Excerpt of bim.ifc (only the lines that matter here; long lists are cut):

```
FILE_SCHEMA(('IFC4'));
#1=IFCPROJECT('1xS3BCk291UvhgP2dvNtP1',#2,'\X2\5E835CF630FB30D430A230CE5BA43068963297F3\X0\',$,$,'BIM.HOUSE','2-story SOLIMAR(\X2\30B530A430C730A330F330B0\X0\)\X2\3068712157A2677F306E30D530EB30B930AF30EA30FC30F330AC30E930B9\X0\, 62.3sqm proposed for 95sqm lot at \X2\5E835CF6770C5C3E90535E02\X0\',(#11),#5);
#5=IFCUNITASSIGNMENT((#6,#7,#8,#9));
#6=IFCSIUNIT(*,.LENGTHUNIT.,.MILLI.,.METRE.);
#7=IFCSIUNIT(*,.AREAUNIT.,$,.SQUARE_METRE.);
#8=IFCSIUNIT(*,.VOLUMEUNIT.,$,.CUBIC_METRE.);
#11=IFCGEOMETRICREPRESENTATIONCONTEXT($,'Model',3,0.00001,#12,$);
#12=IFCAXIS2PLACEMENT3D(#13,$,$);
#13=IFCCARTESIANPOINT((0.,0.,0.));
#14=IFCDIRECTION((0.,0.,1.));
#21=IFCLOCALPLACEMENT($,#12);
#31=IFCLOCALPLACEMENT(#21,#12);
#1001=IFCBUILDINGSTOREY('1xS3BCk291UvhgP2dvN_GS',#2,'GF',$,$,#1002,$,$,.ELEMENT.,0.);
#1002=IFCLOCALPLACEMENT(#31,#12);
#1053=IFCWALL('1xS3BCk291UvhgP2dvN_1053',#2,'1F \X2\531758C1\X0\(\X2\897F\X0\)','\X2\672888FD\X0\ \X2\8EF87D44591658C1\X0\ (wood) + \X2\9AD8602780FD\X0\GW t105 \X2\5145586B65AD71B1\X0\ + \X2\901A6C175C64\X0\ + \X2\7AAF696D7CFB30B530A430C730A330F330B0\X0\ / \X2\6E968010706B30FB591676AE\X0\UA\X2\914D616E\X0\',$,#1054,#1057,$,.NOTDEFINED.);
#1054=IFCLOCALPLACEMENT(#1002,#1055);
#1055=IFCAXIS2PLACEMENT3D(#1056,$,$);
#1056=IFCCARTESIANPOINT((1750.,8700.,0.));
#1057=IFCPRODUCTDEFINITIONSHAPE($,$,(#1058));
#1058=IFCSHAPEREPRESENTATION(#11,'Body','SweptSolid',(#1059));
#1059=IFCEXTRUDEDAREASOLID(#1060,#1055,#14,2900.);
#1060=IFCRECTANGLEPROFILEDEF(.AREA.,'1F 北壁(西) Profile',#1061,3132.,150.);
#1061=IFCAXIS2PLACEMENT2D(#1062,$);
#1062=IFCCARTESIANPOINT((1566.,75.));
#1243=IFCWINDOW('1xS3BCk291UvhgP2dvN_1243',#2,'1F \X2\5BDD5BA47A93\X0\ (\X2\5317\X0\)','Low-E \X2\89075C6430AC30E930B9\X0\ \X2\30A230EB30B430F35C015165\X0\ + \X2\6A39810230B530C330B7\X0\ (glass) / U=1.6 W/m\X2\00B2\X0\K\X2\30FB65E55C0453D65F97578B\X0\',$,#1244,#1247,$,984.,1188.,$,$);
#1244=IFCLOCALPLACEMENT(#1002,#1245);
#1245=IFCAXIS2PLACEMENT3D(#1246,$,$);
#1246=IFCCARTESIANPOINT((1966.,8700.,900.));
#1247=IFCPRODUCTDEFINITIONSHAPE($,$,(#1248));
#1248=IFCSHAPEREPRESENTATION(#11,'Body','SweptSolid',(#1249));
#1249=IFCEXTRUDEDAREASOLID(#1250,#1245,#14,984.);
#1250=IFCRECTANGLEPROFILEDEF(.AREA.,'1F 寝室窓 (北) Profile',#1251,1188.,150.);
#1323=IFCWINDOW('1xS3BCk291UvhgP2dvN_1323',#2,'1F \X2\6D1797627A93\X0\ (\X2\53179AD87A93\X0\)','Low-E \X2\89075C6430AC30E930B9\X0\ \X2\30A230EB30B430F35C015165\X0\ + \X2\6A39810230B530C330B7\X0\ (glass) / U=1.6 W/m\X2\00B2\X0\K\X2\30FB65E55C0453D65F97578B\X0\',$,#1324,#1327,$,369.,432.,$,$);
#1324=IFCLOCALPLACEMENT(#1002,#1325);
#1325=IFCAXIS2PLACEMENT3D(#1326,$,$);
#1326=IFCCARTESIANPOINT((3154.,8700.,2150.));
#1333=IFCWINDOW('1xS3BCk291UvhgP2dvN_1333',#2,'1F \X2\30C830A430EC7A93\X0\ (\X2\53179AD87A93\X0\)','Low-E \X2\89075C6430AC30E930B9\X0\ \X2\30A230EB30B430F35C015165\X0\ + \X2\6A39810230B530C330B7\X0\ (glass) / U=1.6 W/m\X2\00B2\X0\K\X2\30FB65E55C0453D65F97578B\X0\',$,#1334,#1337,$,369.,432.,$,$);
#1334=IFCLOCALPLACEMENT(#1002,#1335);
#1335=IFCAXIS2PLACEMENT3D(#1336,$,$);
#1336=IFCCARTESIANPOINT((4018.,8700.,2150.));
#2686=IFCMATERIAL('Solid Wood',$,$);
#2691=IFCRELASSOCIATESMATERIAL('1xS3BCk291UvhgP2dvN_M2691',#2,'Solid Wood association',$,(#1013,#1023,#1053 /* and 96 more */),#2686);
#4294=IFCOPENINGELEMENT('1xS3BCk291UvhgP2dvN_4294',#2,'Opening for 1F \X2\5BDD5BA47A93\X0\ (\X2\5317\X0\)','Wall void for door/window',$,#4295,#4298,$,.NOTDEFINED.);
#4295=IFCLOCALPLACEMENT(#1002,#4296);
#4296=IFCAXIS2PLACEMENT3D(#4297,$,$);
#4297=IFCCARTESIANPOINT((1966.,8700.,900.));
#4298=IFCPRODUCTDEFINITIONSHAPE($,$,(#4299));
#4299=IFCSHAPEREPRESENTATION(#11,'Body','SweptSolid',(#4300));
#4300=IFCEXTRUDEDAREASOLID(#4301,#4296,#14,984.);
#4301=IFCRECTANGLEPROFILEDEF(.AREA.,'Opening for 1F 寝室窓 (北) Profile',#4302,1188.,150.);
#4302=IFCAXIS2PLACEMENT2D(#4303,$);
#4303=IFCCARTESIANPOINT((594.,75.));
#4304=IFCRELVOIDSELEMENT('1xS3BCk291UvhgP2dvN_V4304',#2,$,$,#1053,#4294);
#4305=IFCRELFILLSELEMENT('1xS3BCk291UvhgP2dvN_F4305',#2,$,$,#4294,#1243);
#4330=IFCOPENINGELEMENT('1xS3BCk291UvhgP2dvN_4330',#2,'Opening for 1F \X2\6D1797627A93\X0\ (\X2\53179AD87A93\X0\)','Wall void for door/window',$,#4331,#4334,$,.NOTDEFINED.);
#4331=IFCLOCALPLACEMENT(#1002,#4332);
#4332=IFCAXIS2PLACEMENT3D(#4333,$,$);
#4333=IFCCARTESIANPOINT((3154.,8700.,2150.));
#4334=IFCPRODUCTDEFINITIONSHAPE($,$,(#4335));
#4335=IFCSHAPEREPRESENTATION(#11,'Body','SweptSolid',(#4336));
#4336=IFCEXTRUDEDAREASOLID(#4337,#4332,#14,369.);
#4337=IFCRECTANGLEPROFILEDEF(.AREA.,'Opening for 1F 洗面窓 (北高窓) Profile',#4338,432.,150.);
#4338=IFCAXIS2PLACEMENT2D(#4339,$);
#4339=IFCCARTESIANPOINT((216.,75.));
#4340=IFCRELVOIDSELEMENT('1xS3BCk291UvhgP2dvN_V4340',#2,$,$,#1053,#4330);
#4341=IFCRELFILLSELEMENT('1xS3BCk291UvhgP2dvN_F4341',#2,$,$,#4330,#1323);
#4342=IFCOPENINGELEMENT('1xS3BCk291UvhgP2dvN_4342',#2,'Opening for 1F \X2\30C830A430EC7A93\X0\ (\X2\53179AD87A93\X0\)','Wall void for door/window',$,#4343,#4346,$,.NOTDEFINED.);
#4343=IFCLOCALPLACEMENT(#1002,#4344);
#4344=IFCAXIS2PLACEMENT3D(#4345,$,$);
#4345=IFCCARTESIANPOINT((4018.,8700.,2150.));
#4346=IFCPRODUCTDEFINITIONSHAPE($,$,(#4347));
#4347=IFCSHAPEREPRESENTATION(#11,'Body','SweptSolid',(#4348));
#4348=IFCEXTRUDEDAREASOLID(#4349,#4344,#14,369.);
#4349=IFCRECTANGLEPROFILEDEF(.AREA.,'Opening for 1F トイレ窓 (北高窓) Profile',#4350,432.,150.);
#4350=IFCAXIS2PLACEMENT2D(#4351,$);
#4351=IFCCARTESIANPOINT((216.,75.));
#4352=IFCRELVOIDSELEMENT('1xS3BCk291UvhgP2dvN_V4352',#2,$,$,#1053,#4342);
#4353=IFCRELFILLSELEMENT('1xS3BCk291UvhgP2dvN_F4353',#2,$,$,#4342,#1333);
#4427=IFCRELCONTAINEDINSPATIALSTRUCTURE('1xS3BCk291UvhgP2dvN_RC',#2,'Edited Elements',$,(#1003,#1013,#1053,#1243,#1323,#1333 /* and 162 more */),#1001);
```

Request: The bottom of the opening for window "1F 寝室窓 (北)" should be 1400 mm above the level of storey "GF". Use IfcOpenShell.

```python
import numpy as np
import ifcopenshell
import ifcopenshell.api.geometry
import ifcopenshell.geom
import ifcopenshell.util.element
import ifcopenshell.util.placement
import ifcopenshell.util.shape
import ifcopenshell.util.unit

model = ifcopenshell.open("bim.ifc")
unit_scale = ifcopenshell.util.unit.calculate_unit_scale(model)

window = model.by_guid("1xS3BCk291UvhgP2dvN_1243")
opening = window.FillsVoids[0].RelatingOpeningElement
storey = ifcopenshell.util.element.get_container(window, ifc_class="IfcBuildingStorey")
level = ifcopenshell.util.placement.get_local_placement(storey.ObjectPlacement)[2, 3]

# The opening's origin need not be at the sill, so measure its lowest point.
shape = ifcopenshell.geom.create_shape(ifcopenshell.geom.settings(), opening)
bottom = ifcopenshell.util.shape.get_shape_bottom_elevation(shape, shape.geometry) / unit_scale
dz = level + 1.4 / unit_scale - bottom

shift = np.array([0.0, 0.0, dz])
# The window is not placed relative to its opening, so move both.
for product in (opening, window):
    matrix = ifcopenshell.util.placement.get_local_placement(product.ObjectPlacement)
    matrix[:3, 3] += shift
    ifcopenshell.api.geometry.edit_object_placement(model, product=product, matrix=matrix, is_si=False)

print(f"moved by {dz * unit_scale:+.3f} m")

model.write("bim-out.ifc")
```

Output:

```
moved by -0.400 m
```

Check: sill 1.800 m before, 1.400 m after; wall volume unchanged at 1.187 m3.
